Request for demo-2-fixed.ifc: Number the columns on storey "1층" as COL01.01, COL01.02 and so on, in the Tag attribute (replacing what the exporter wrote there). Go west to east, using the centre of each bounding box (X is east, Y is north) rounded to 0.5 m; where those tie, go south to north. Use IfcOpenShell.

First a look at what the model holds.

```python
import ifcopenshell
import ifcopenshell.util.element
import ifcopenshell.util.placement

model = ifcopenshell.open("demo-2-fixed.ifc")
print(model.schema)
storey = next(s for s in model.by_type("IfcBuildingStorey") if s.Name == "1층")
columns = [e for e in ifcopenshell.util.element.get_decomposition(storey) if e.is_a("IfcColumn")]
for e in sorted(columns, key=lambda e: e.id()):
    origin = ifcopenshell.util.placement.get_local_placement(e.ObjectPlacement)[:3, 3]
    print(e.id(), e.Tag, e.Name, origin.round(2) + 0.0, sep=" | ")
```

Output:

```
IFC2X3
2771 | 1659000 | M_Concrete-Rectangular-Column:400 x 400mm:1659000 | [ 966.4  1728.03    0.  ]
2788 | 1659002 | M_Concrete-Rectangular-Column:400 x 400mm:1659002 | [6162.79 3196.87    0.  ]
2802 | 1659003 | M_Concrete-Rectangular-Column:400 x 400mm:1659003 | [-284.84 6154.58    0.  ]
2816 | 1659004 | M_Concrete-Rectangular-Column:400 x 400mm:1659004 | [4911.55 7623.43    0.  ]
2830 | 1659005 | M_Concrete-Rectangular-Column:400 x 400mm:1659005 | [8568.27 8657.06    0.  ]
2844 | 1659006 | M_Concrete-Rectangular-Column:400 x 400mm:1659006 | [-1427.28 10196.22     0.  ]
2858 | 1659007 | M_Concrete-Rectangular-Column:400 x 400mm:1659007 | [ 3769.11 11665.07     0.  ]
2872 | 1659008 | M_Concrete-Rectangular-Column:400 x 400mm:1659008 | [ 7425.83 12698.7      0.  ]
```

```python
import ifcopenshell
import ifcopenshell.geom
import ifcopenshell.util.element
import ifcopenshell.util.shape

model = ifcopenshell.open("demo-2-fixed.ifc")
settings = ifcopenshell.geom.settings()
settings.set("use-world-coords", True)


def centre(element):
    shape = ifcopenshell.geom.create_shape(settings, element)
    return ifcopenshell.util.shape.get_bbox_centroid(shape.geometry)


storey = next(s for s in model.by_type("IfcBuildingStorey") if s.Name == "1층")
columns = [e for e in ifcopenshell.util.element.get_decomposition(storey) if e.is_a("IfcColumn")]

# Insertion points can sit at a corner or the storey origin, so sort by the geometry (in metres).
centres = {e: centre(e) for e in columns}
columns.sort(key=lambda e: (round(centres[e][0] / 0.5), centres[e][1]))

for i, e in enumerate(columns, start=1):
    number = f"COL01.{i:02d}"
    e.Tag = number
    print(e.id(), number)

model.write("demo-2-fixed-out.ifc")
```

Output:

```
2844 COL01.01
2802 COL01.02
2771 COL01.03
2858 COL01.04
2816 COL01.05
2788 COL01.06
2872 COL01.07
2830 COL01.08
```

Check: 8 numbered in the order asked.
